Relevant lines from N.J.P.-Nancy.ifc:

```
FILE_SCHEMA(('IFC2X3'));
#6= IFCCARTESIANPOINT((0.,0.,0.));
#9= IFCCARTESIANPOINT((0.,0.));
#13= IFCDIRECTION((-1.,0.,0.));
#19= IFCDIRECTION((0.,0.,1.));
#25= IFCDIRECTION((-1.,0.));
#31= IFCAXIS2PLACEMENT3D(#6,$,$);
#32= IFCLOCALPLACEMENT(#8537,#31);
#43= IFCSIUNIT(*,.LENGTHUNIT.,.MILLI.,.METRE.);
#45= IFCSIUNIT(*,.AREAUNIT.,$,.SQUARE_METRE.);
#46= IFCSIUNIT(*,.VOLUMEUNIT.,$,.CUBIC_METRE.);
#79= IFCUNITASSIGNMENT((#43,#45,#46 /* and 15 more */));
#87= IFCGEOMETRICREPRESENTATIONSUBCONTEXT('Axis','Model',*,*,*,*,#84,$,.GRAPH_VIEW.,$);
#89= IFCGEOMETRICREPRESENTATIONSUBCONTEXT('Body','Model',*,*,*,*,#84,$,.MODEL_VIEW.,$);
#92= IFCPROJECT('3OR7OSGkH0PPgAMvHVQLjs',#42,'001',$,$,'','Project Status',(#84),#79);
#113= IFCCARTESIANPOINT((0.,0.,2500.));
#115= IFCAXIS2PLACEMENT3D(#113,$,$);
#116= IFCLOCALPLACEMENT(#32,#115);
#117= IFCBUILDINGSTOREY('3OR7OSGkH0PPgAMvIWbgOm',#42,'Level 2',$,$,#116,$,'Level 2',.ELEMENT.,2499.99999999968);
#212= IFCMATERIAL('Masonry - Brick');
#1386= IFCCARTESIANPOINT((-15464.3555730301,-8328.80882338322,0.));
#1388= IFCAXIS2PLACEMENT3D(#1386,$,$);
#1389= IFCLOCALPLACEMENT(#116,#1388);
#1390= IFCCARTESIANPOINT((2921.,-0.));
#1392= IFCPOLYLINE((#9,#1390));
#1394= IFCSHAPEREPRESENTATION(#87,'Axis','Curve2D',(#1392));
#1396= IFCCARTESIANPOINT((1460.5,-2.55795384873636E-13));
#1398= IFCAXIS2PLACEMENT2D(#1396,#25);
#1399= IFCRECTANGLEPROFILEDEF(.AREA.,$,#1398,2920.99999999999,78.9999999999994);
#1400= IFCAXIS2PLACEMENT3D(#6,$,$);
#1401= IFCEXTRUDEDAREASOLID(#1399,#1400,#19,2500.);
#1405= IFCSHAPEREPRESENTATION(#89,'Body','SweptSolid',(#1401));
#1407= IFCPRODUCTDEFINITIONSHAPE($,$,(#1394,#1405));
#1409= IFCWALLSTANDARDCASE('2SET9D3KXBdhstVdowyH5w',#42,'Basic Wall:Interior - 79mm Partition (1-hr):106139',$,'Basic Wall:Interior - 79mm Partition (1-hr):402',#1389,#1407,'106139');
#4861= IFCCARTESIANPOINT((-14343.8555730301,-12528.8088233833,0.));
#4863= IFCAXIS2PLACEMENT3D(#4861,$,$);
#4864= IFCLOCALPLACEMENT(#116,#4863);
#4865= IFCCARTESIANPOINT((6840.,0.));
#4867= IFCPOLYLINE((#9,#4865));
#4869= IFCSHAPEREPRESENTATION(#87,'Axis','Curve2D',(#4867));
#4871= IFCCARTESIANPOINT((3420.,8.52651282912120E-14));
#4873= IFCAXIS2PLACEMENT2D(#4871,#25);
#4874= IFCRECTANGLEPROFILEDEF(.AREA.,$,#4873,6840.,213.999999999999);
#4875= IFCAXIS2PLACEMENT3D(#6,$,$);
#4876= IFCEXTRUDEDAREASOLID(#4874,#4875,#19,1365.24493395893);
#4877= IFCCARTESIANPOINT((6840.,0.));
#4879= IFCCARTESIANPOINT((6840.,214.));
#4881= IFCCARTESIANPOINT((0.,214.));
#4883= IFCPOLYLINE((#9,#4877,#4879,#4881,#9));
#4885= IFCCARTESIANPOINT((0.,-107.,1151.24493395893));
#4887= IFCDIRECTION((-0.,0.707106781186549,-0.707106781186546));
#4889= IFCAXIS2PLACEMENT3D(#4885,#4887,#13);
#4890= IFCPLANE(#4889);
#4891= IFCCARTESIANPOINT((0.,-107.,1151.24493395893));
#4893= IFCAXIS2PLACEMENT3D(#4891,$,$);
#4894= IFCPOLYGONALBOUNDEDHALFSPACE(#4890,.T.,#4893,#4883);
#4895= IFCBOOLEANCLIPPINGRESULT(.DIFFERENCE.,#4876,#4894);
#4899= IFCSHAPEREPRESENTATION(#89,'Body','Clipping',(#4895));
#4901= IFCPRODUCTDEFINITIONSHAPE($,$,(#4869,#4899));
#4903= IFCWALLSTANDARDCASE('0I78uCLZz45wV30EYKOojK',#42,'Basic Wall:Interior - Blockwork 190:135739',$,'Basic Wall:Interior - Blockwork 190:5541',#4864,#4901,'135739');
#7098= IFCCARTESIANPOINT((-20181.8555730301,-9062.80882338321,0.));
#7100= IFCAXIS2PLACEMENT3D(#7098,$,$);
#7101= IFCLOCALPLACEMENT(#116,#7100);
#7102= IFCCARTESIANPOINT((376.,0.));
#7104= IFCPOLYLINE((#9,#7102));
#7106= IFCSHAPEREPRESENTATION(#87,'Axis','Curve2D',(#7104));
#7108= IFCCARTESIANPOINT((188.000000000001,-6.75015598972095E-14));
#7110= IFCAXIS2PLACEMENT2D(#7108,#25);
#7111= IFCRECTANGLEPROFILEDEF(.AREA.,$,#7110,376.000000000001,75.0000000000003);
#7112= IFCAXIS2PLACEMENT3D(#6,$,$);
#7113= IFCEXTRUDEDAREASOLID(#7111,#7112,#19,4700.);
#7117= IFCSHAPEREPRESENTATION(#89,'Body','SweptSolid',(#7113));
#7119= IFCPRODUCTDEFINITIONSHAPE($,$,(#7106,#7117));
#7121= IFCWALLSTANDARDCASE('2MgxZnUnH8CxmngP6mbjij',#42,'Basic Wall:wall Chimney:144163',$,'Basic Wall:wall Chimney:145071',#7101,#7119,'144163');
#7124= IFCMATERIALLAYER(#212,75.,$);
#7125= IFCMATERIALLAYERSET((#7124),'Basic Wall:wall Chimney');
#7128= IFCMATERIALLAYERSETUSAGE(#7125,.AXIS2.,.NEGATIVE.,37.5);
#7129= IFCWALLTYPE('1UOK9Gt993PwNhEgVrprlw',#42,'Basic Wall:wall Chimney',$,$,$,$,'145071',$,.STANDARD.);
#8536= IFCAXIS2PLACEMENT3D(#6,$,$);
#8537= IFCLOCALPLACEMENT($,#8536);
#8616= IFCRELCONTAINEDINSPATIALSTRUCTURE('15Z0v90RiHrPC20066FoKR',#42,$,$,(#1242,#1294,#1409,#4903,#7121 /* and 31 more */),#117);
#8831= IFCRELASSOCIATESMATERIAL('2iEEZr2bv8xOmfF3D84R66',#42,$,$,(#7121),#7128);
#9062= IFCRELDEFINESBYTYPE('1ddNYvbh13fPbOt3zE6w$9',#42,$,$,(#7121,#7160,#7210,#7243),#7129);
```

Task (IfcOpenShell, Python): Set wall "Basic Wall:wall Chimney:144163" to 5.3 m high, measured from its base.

```python
import ifcopenshell
import ifcopenshell.geom
import ifcopenshell.util.representation
import ifcopenshell.util.shape
import ifcopenshell.util.unit

model = ifcopenshell.open("N.J.P.-Nancy.ifc")
unit_scale = ifcopenshell.util.unit.calculate_unit_scale(model)
settings = ifcopenshell.geom.settings()


def volume(element):
    """Net volume in cubic metres, openings subtracted."""
    shape = ifcopenshell.geom.create_shape(settings, element)
    return ifcopenshell.util.shape.get_volume(shape.geometry)


wall = model.by_id(7121)
before = volume(wall)

body = ifcopenshell.util.representation.get_representation(wall, "Model", "Body")
solid = body.Items[0]
old_height = solid.Depth
solid.Depth = 5.3 / unit_scale
after = volume(wall)

print(f"height {old_height:g} -> {solid.Depth:g}, volume {before:.3f} -> {after:.3f} m3")

model.write("N.J.P.-Nancy_v2.ifc")
```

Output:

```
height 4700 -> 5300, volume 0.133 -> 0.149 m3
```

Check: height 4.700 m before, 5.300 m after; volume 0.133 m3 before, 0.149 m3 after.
